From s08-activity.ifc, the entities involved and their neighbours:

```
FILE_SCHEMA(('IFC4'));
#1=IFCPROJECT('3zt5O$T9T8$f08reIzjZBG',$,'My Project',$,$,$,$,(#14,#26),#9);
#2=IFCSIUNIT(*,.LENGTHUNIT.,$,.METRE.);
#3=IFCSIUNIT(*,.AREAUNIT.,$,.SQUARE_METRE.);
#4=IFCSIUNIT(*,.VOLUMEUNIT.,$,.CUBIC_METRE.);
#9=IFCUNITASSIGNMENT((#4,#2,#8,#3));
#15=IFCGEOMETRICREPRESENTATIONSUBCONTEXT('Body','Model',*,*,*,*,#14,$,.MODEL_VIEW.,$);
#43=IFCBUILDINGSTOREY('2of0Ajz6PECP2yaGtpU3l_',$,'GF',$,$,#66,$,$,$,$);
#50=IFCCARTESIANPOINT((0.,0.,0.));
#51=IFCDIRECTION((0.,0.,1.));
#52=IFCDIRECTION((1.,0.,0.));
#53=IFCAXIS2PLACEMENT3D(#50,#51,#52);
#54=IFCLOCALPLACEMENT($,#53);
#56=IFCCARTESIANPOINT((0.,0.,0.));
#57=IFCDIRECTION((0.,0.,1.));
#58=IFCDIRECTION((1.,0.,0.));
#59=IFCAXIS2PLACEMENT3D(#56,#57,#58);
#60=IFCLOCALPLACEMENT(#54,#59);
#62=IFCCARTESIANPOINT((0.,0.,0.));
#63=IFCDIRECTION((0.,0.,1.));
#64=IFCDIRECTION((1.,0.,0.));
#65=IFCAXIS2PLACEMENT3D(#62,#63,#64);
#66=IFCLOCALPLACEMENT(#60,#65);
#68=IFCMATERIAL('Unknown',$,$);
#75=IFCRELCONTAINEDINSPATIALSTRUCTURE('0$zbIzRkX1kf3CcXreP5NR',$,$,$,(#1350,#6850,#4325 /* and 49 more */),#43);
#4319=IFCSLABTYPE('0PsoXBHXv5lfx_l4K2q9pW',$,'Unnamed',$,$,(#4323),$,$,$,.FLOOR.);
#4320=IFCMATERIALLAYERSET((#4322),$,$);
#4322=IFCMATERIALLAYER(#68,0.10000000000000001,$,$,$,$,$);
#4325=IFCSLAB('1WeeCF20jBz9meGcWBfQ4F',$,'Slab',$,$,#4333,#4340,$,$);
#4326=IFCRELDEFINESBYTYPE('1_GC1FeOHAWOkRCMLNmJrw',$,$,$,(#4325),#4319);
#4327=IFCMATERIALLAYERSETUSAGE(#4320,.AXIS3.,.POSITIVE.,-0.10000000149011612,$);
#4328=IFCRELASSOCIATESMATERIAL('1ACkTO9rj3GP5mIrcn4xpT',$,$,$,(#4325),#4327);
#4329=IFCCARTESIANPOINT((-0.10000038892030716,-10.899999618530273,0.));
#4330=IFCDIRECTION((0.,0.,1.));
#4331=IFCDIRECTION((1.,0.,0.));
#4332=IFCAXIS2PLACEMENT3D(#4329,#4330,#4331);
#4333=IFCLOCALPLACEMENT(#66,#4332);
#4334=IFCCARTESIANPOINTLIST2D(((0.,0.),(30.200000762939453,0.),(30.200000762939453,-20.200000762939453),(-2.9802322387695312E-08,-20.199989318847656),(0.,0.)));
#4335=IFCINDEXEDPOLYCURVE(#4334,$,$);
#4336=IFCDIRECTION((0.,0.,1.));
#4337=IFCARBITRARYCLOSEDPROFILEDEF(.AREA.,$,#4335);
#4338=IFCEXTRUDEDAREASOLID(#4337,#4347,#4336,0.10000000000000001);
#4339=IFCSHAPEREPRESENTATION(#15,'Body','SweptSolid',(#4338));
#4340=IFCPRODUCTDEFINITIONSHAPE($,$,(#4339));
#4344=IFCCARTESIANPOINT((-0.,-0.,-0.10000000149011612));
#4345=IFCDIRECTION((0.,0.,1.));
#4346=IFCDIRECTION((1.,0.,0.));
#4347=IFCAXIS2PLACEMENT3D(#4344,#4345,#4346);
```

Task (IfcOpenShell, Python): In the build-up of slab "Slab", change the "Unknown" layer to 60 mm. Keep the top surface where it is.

```python
import ifcopenshell
import ifcopenshell.util.element
import ifcopenshell.util.representation

model = ifcopenshell.open("s08-activity.ifc")

layer_set = model.by_id(4320)
layer = next(l for l in layer_set.MaterialLayers if l.Material and l.Material.Name == "Unknown")
change = 0.06 - layer.LayerThickness
layer.LayerThickness += change

# Geometry does not follow the layer set by itself.
slabs = [e for e in ifcopenshell.util.element.get_elements_by_material(model, layer_set) if e.is_a("IfcSlab")]
for slab in sorted(slabs, key=lambda e: e.id()):
    body = ifcopenshell.util.representation.get_representation(slab, "Model", "Body")
    solid = body.Items[0]
    old_depth = solid.Depth
    solid.Depth += change
    # Extruded upwards: lower the start of the extrusion so the top stays.
    x, y, z = solid.Position.Location.Coordinates
    solid.Position.Location = model.createIfcCartesianPoint((x, y, z - change))
    print(slab.id(), f"{old_depth:g} -> {solid.Depth:g}")

# The layers are counted up from the underside, which has moved.
for usage in {ifcopenshell.util.element.get_material(slab) for slab in slabs}:
    usage.OffsetFromReferenceLine -= change

model.write("s08-activity_edited.ifc")
```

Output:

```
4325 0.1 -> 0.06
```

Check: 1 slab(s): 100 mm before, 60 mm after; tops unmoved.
